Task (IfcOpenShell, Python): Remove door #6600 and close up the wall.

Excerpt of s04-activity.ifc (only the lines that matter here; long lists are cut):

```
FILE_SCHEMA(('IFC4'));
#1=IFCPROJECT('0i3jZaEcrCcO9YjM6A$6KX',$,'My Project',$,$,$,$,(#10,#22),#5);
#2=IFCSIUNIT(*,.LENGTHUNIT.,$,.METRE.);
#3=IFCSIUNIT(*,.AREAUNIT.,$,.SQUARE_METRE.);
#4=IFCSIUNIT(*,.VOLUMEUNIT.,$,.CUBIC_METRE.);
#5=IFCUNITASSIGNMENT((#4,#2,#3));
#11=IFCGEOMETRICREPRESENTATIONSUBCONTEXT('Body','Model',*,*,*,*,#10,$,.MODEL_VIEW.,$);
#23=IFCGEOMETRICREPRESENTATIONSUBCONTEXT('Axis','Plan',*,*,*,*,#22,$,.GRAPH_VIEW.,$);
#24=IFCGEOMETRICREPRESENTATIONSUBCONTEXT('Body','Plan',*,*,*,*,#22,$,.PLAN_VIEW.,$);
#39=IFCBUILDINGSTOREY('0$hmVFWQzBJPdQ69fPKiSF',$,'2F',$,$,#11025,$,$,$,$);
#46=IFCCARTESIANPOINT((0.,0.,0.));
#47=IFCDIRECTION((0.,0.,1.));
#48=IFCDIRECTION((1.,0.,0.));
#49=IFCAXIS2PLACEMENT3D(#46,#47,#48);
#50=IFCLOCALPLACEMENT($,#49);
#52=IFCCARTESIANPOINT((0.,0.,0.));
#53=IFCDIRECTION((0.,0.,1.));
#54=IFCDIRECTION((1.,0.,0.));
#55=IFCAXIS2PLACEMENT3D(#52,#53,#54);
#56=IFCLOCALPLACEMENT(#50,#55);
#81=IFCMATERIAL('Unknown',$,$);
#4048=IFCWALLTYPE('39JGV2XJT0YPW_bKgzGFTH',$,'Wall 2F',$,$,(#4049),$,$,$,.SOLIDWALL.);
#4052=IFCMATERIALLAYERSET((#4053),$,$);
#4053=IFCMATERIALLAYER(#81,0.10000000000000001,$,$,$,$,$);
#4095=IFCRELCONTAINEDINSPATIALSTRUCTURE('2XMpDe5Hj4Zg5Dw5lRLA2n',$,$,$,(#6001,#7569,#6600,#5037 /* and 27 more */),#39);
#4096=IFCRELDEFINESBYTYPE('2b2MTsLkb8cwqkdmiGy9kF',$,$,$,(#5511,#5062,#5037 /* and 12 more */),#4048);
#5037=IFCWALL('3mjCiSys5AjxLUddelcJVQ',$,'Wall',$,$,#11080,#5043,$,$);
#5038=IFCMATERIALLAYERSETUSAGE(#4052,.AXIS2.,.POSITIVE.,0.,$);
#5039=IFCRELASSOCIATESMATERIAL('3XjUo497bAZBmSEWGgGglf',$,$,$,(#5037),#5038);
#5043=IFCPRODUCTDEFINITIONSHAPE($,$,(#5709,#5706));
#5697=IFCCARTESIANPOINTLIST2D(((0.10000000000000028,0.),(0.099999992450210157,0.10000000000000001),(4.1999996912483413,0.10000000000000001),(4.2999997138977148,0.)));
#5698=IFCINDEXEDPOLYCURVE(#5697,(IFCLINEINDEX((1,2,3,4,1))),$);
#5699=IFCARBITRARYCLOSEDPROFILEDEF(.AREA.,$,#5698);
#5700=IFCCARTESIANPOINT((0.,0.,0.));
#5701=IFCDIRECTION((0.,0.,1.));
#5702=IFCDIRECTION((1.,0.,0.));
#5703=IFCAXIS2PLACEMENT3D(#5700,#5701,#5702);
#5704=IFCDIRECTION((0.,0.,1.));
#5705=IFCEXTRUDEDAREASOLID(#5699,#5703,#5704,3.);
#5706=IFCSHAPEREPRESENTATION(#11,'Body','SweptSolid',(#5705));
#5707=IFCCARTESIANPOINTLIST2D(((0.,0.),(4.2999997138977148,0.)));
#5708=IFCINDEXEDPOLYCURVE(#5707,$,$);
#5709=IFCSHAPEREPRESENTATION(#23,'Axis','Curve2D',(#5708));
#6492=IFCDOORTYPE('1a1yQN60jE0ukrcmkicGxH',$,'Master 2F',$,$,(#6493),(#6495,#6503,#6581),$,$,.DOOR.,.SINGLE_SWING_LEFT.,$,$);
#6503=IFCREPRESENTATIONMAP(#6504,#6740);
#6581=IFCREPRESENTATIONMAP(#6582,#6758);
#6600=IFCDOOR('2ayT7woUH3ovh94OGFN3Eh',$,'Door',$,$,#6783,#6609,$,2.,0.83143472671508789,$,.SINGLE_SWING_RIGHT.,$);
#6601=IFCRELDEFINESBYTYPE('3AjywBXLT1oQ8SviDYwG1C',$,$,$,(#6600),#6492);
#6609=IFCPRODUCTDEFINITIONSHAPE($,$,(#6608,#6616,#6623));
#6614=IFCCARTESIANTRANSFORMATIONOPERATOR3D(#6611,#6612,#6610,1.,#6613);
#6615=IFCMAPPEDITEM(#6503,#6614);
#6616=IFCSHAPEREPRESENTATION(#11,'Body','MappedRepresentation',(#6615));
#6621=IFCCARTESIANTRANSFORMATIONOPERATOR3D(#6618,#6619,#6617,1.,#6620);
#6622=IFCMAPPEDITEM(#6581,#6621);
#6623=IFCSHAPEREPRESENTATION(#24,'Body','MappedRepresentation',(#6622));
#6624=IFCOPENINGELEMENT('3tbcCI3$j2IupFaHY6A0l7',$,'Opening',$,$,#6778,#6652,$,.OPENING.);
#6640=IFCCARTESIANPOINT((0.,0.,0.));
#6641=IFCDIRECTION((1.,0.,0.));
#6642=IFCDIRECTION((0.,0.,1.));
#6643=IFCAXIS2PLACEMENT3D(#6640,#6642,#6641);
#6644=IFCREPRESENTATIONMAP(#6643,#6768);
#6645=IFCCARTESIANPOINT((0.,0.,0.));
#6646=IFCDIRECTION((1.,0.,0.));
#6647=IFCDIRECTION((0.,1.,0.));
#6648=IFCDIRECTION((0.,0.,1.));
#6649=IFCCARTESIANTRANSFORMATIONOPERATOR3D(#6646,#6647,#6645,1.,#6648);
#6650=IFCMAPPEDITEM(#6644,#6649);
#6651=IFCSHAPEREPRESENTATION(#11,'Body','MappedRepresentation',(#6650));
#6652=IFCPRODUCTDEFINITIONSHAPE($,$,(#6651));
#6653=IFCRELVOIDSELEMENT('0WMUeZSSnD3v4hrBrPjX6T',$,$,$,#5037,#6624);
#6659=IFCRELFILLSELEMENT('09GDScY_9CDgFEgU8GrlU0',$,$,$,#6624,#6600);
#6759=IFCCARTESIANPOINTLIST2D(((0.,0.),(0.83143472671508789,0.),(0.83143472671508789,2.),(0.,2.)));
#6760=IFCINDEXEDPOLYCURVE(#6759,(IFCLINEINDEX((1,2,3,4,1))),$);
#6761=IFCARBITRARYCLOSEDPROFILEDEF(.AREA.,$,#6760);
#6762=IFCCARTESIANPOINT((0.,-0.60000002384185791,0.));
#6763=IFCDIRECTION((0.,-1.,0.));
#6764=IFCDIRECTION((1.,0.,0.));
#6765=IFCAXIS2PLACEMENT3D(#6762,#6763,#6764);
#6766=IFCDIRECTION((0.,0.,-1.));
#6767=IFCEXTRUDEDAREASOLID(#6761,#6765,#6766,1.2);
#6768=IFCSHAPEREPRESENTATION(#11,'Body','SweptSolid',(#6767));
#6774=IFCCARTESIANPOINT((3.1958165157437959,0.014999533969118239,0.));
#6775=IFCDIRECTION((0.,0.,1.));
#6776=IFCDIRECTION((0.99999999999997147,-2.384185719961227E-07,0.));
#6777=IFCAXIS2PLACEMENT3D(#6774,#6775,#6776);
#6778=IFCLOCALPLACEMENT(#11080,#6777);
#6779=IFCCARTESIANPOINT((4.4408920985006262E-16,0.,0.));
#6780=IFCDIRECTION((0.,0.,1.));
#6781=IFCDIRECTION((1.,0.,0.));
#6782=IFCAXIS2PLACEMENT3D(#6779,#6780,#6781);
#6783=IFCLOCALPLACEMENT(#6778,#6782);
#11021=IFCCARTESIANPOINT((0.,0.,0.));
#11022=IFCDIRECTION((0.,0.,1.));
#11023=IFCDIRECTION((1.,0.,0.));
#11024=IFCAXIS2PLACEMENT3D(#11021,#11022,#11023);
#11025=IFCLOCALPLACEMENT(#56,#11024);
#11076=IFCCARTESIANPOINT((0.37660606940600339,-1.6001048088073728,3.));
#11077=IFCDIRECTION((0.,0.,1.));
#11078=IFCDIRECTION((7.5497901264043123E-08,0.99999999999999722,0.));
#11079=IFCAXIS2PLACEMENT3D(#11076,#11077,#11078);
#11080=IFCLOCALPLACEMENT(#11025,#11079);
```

```python
import ifcopenshell
import ifcopenshell.api.feature
import ifcopenshell.api.root
import ifcopenshell.geom
import ifcopenshell.util.shape

model = ifcopenshell.open("s04-activity.ifc")
settings = ifcopenshell.geom.settings()


def volume(element):
    """Net volume in cubic metres, openings subtracted."""
    shape = ifcopenshell.geom.create_shape(settings, element)
    return ifcopenshell.util.shape.get_volume(shape.geometry)


door = model.by_guid("2ayT7woUH3ovh94OGFN3Eh")
opening = door.FillsVoids[0].RelatingOpeningElement
wall = opening.VoidsElements[0].RelatingBuildingElement
before = volume(wall)

ifcopenshell.api.root.remove_product(model, product=door)
ifcopenshell.api.feature.remove_feature(model, feature=opening)

after = volume(wall)

print(f"wall volume {before:.3f} -> {after:.3f} m3")

model.write("s04-activity_edited.ifc")
```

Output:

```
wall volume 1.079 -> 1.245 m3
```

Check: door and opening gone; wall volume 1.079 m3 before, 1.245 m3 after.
